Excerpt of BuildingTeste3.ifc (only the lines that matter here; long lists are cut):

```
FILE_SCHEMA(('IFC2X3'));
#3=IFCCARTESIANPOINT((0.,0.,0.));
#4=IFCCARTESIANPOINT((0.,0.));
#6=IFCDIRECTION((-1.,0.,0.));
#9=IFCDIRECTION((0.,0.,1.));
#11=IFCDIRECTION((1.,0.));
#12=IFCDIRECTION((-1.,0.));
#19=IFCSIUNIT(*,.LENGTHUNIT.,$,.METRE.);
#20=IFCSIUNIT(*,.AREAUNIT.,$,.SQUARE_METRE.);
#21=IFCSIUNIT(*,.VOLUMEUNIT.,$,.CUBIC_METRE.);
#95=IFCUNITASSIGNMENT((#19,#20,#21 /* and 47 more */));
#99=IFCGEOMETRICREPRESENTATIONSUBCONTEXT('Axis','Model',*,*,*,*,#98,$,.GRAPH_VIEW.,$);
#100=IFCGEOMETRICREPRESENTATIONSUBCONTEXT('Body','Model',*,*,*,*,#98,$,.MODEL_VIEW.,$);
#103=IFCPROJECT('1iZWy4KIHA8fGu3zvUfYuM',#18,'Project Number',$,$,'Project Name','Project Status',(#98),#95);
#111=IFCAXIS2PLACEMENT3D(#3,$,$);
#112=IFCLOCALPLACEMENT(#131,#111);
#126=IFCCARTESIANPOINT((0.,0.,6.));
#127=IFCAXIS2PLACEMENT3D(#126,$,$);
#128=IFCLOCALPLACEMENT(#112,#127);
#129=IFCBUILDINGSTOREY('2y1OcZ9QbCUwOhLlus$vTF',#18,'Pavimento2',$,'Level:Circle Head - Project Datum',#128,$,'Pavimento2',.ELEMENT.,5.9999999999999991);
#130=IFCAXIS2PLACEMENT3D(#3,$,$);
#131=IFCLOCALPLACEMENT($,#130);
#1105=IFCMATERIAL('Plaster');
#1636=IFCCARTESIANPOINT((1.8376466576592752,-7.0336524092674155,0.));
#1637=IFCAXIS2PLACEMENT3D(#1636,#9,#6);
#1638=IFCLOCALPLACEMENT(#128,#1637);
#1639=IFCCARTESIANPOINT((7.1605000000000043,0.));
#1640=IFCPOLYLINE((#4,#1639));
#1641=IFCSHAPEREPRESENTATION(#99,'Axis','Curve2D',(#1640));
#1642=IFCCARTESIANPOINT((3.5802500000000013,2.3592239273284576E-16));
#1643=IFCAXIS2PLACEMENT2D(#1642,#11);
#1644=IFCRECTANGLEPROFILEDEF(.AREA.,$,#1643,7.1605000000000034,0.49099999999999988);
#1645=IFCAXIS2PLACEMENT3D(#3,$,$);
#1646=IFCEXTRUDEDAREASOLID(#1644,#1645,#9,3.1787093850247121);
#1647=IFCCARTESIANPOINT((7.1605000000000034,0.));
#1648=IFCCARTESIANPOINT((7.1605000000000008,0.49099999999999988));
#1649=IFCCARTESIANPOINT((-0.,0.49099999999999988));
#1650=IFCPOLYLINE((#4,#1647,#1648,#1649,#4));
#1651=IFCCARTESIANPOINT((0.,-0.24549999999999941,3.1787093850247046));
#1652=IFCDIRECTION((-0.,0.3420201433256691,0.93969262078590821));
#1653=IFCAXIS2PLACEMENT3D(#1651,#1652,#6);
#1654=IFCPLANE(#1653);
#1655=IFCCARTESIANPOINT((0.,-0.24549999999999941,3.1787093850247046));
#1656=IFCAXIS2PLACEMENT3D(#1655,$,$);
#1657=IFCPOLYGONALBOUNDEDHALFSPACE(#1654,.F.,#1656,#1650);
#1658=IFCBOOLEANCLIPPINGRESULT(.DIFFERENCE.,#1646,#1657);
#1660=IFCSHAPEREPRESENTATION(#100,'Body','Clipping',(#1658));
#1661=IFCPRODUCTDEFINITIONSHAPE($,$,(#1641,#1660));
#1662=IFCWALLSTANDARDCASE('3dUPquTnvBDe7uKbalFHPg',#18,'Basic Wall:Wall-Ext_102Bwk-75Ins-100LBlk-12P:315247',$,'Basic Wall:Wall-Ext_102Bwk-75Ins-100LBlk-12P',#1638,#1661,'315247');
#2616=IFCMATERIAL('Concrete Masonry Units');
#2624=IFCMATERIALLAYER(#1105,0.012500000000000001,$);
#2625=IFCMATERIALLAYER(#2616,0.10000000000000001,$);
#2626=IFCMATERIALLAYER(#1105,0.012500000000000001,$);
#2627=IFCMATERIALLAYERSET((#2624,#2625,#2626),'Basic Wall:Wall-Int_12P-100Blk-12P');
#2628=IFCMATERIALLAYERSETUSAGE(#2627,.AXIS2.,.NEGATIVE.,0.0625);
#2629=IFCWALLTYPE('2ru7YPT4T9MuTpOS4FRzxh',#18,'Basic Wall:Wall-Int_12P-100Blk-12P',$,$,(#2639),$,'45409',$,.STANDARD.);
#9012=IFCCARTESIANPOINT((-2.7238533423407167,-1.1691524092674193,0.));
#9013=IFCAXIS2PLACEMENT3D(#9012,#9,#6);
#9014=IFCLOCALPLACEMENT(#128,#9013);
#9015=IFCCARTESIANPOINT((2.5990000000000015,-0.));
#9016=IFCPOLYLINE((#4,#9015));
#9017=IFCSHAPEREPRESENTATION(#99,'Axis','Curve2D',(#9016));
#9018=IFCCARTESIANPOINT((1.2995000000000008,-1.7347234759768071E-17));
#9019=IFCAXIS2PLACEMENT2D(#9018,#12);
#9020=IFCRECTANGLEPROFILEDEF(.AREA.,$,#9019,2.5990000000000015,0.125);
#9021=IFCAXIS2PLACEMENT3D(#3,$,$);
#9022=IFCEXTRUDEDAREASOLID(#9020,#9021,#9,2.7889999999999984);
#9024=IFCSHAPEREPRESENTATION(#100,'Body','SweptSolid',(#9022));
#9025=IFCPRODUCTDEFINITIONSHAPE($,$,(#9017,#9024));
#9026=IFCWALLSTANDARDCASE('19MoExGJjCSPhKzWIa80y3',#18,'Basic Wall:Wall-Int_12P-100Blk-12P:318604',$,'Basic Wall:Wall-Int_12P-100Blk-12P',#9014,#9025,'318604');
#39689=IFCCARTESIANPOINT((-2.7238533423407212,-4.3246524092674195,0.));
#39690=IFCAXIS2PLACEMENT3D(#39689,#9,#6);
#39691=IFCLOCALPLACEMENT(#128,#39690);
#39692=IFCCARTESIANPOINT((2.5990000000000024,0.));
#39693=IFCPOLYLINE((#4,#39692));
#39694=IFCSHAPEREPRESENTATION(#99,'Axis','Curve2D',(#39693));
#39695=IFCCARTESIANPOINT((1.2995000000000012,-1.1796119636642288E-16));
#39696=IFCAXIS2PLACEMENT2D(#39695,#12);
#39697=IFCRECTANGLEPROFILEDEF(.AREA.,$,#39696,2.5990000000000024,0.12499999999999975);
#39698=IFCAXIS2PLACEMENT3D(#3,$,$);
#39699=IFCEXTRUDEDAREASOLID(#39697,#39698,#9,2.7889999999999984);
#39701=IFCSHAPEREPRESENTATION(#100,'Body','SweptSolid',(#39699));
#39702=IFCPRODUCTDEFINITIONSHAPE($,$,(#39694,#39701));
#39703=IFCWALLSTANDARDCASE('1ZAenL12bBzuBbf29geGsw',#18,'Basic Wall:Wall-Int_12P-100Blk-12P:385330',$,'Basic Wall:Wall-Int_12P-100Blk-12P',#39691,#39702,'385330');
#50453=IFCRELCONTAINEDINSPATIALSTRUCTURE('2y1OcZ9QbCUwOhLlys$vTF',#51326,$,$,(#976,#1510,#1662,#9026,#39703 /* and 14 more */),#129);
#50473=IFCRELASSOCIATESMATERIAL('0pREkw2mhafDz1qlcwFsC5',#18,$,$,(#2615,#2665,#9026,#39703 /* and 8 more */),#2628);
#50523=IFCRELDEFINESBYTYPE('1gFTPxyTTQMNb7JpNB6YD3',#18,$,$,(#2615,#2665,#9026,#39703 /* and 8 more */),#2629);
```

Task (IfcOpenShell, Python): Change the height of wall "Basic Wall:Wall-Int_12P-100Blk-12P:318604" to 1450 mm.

```python
import ifcopenshell
import ifcopenshell.geom
import ifcopenshell.util.representation
import ifcopenshell.util.shape

model = ifcopenshell.open("BuildingTeste3.ifc")
settings = ifcopenshell.geom.settings()


def volume(element):
    """Net volume in cubic metres, openings subtracted."""
    shape = ifcopenshell.geom.create_shape(settings, element)
    return ifcopenshell.util.shape.get_volume(shape.geometry)


wall = model.by_guid("19MoExGJjCSPhKzWIa80y3")
before = volume(wall)

body = ifcopenshell.util.representation.get_representation(wall, "Model", "Body")
solid = body.Items[0]
old_height = solid.Depth
solid.Depth = 1.45
after = volume(wall)

print(f"height {old_height:g} -> {solid.Depth:g}, volume {before:.3f} -> {after:.3f} m3")

model.write("BuildingTeste3_rev.ifc")
```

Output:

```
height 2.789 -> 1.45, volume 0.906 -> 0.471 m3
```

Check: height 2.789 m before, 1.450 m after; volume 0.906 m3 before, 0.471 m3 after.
